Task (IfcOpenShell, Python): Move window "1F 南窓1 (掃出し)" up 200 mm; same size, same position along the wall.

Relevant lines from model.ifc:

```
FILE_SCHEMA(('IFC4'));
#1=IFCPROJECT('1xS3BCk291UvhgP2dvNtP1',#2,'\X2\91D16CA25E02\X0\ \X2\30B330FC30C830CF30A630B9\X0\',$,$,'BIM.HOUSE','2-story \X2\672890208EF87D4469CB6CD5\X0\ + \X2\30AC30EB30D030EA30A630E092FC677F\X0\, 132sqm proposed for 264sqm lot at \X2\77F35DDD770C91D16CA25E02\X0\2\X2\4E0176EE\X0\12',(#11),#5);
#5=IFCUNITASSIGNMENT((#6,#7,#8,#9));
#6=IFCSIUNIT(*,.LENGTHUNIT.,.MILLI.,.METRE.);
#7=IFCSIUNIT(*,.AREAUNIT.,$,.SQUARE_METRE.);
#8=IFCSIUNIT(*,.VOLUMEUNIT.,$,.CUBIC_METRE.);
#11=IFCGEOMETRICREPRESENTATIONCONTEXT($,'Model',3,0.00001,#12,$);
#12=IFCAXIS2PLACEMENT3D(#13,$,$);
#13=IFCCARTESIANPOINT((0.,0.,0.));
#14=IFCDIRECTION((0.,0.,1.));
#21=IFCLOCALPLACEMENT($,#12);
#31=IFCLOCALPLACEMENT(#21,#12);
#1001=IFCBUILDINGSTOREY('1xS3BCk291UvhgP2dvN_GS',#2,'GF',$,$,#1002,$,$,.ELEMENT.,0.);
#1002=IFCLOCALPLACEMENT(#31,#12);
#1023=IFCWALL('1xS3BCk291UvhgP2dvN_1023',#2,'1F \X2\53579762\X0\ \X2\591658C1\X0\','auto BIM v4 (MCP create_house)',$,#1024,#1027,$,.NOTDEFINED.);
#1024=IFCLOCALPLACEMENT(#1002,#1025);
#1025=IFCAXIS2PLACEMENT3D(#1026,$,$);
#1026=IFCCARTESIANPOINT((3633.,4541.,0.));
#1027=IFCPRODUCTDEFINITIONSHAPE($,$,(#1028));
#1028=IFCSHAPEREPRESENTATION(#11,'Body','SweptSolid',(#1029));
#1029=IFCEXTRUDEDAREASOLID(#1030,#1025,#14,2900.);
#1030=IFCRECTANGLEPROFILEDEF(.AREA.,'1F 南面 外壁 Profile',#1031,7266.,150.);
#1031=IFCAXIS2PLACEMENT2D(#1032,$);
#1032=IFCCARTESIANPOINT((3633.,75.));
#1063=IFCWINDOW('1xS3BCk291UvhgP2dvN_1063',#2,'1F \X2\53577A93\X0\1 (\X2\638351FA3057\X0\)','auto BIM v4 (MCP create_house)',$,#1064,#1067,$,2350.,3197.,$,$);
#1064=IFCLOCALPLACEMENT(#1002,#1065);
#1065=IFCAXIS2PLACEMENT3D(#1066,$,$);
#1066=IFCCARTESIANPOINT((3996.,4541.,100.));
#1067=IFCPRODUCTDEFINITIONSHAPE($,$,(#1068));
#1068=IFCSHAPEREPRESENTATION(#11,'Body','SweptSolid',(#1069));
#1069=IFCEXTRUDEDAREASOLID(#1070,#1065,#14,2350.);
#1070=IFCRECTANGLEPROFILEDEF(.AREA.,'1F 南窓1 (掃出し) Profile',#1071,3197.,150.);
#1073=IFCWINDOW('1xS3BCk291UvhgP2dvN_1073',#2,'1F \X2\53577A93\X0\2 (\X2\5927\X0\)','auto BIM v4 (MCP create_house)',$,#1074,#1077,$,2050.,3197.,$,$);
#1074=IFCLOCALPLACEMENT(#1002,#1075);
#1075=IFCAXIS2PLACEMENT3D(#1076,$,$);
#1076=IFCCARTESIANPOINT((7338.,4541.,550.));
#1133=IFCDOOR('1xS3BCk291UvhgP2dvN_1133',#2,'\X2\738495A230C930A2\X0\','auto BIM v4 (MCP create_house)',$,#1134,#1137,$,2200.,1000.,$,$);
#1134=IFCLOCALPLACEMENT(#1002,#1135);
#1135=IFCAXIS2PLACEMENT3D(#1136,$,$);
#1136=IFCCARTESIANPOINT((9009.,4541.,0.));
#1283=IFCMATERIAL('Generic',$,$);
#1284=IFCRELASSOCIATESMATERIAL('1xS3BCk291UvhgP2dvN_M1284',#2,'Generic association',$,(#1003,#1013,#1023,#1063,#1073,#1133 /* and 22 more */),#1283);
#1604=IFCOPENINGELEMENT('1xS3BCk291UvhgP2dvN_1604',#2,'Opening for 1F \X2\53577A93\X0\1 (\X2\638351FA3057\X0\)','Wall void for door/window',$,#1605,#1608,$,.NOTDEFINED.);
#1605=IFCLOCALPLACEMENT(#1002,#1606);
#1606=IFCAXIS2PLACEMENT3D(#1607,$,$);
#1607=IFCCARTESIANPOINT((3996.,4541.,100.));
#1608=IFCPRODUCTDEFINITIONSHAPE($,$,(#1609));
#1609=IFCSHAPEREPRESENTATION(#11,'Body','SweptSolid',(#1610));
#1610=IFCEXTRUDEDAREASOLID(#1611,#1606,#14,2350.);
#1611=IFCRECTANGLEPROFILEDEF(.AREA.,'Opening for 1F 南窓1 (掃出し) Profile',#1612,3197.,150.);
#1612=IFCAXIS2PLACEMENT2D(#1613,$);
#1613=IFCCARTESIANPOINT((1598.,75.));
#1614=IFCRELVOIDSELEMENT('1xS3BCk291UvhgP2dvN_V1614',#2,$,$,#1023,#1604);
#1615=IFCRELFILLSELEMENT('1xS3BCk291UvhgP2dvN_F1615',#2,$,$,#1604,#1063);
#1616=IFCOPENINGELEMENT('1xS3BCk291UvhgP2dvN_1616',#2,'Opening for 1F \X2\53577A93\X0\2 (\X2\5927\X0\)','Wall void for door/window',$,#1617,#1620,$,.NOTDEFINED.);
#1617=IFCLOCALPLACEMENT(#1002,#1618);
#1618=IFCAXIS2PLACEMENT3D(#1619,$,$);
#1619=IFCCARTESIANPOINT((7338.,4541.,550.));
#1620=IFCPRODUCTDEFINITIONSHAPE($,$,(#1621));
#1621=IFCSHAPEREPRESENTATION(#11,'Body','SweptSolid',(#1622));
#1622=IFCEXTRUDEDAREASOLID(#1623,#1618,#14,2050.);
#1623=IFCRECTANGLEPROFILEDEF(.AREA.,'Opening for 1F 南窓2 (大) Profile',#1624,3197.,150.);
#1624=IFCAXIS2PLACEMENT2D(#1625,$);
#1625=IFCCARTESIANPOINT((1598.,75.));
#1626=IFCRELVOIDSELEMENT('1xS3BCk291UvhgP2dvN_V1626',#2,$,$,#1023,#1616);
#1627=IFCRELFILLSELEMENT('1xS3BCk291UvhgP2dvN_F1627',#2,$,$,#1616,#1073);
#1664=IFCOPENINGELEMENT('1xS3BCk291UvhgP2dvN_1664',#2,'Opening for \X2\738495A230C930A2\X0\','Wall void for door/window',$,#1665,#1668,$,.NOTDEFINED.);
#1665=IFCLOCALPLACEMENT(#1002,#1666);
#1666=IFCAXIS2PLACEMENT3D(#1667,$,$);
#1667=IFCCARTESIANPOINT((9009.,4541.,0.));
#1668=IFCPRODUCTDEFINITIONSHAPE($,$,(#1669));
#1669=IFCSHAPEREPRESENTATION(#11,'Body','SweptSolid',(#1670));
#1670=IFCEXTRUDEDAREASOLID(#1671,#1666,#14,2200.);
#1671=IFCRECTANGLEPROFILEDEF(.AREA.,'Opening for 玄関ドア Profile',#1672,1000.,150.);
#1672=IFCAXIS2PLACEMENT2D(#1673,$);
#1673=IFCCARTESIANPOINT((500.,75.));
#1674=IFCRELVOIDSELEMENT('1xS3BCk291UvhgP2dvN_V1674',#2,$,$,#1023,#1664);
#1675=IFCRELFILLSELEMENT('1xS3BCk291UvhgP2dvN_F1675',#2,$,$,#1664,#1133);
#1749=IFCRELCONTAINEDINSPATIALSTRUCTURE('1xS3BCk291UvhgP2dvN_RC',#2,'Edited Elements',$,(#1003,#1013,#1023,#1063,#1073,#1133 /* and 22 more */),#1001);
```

```python
import numpy as np
import ifcopenshell
import ifcopenshell.api.geometry
import ifcopenshell.util.placement
import ifcopenshell.util.unit

model = ifcopenshell.open("model.ifc")
unit_scale = ifcopenshell.util.unit.calculate_unit_scale(model)

window = model.by_id(1063)
opening = window.FillsVoids[0].RelatingOpeningElement
dz = 200.0

shift = np.array([0.0, 0.0, dz])
# The window is not placed relative to its opening, so move both.
for product in (opening, window):
    matrix = ifcopenshell.util.placement.get_local_placement(product.ObjectPlacement)
    matrix[:3, 3] += shift
    ifcopenshell.api.geometry.edit_object_placement(model, product=product, matrix=matrix, is_si=False)

print(f"moved by {dz * unit_scale:+.3f} m")

model.write("model-out.ifc")
```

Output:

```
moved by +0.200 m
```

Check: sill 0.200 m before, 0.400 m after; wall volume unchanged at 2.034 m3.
